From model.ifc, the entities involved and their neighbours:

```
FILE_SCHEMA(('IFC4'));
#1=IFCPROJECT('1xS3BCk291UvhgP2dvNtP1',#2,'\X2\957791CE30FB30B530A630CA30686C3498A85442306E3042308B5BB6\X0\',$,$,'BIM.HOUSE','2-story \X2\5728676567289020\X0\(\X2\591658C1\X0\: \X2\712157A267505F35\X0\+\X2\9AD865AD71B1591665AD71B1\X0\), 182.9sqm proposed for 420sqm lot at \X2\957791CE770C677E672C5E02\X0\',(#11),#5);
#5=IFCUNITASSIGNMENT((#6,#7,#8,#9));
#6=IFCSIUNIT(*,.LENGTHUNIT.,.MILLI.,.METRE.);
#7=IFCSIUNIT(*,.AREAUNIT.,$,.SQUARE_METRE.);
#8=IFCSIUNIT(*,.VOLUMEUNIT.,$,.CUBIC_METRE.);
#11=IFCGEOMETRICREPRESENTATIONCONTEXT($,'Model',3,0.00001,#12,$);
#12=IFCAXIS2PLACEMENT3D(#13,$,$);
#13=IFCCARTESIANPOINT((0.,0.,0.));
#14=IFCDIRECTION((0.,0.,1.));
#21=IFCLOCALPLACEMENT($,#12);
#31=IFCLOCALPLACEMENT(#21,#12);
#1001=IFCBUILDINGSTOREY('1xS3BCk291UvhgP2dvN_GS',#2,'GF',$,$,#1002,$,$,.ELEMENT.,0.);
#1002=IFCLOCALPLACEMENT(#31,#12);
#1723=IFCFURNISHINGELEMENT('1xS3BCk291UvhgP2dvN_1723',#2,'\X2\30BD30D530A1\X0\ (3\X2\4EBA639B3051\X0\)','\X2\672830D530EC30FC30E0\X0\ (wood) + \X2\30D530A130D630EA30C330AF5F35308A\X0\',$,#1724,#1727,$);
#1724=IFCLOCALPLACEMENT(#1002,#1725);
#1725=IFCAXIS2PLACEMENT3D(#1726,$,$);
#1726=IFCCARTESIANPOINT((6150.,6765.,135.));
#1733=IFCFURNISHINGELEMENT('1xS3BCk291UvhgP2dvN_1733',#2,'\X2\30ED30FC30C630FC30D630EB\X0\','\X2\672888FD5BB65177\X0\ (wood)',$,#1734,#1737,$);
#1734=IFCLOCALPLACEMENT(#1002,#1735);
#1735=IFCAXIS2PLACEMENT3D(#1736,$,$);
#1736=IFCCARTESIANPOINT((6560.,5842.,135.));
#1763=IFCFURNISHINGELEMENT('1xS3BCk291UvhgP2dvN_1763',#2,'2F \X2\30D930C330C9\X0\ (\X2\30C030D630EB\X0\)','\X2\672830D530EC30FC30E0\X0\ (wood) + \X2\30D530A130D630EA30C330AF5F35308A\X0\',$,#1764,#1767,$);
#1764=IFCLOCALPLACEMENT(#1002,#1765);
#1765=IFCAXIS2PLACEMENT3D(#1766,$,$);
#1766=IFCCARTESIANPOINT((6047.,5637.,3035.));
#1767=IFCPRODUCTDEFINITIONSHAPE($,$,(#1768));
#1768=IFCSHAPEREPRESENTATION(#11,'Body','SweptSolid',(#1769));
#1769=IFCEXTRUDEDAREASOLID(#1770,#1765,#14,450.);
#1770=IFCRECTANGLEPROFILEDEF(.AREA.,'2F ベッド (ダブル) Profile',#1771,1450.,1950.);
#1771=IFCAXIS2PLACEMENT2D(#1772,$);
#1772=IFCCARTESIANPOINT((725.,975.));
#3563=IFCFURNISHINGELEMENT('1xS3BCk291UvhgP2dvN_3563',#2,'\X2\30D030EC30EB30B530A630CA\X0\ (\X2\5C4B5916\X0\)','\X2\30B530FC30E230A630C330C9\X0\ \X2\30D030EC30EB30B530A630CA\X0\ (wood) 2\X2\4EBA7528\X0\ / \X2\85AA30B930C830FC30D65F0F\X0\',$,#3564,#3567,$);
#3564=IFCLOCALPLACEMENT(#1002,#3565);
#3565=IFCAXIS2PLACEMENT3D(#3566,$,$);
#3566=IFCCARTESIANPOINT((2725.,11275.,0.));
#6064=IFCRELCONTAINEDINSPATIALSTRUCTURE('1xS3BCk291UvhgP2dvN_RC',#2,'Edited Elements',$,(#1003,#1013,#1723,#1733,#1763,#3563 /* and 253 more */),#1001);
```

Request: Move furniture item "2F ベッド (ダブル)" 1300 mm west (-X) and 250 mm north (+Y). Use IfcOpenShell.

```python
import ifcopenshell
import ifcopenshell.api.geometry
import ifcopenshell.util.placement
import ifcopenshell.util.unit

model = ifcopenshell.open("model.ifc")
unit_scale = ifcopenshell.util.unit.calculate_unit_scale(model)

item = model.by_guid("1xS3BCk291UvhgP2dvN_1763")
matrix = ifcopenshell.util.placement.get_local_placement(item.ObjectPlacement)
matrix[0, 3] -= 1.3 / unit_scale
matrix[1, 3] += 0.25 / unit_scale
ifcopenshell.api.geometry.edit_object_placement(model, product=item, matrix=matrix, is_si=False)

print(ifcopenshell.util.placement.get_local_placement(item.ObjectPlacement).round(3) + 0.0)

model.write("model-out.ifc")
```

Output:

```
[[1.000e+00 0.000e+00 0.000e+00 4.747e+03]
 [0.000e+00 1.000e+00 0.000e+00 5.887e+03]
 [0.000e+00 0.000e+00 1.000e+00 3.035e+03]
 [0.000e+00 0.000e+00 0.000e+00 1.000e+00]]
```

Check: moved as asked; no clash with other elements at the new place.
